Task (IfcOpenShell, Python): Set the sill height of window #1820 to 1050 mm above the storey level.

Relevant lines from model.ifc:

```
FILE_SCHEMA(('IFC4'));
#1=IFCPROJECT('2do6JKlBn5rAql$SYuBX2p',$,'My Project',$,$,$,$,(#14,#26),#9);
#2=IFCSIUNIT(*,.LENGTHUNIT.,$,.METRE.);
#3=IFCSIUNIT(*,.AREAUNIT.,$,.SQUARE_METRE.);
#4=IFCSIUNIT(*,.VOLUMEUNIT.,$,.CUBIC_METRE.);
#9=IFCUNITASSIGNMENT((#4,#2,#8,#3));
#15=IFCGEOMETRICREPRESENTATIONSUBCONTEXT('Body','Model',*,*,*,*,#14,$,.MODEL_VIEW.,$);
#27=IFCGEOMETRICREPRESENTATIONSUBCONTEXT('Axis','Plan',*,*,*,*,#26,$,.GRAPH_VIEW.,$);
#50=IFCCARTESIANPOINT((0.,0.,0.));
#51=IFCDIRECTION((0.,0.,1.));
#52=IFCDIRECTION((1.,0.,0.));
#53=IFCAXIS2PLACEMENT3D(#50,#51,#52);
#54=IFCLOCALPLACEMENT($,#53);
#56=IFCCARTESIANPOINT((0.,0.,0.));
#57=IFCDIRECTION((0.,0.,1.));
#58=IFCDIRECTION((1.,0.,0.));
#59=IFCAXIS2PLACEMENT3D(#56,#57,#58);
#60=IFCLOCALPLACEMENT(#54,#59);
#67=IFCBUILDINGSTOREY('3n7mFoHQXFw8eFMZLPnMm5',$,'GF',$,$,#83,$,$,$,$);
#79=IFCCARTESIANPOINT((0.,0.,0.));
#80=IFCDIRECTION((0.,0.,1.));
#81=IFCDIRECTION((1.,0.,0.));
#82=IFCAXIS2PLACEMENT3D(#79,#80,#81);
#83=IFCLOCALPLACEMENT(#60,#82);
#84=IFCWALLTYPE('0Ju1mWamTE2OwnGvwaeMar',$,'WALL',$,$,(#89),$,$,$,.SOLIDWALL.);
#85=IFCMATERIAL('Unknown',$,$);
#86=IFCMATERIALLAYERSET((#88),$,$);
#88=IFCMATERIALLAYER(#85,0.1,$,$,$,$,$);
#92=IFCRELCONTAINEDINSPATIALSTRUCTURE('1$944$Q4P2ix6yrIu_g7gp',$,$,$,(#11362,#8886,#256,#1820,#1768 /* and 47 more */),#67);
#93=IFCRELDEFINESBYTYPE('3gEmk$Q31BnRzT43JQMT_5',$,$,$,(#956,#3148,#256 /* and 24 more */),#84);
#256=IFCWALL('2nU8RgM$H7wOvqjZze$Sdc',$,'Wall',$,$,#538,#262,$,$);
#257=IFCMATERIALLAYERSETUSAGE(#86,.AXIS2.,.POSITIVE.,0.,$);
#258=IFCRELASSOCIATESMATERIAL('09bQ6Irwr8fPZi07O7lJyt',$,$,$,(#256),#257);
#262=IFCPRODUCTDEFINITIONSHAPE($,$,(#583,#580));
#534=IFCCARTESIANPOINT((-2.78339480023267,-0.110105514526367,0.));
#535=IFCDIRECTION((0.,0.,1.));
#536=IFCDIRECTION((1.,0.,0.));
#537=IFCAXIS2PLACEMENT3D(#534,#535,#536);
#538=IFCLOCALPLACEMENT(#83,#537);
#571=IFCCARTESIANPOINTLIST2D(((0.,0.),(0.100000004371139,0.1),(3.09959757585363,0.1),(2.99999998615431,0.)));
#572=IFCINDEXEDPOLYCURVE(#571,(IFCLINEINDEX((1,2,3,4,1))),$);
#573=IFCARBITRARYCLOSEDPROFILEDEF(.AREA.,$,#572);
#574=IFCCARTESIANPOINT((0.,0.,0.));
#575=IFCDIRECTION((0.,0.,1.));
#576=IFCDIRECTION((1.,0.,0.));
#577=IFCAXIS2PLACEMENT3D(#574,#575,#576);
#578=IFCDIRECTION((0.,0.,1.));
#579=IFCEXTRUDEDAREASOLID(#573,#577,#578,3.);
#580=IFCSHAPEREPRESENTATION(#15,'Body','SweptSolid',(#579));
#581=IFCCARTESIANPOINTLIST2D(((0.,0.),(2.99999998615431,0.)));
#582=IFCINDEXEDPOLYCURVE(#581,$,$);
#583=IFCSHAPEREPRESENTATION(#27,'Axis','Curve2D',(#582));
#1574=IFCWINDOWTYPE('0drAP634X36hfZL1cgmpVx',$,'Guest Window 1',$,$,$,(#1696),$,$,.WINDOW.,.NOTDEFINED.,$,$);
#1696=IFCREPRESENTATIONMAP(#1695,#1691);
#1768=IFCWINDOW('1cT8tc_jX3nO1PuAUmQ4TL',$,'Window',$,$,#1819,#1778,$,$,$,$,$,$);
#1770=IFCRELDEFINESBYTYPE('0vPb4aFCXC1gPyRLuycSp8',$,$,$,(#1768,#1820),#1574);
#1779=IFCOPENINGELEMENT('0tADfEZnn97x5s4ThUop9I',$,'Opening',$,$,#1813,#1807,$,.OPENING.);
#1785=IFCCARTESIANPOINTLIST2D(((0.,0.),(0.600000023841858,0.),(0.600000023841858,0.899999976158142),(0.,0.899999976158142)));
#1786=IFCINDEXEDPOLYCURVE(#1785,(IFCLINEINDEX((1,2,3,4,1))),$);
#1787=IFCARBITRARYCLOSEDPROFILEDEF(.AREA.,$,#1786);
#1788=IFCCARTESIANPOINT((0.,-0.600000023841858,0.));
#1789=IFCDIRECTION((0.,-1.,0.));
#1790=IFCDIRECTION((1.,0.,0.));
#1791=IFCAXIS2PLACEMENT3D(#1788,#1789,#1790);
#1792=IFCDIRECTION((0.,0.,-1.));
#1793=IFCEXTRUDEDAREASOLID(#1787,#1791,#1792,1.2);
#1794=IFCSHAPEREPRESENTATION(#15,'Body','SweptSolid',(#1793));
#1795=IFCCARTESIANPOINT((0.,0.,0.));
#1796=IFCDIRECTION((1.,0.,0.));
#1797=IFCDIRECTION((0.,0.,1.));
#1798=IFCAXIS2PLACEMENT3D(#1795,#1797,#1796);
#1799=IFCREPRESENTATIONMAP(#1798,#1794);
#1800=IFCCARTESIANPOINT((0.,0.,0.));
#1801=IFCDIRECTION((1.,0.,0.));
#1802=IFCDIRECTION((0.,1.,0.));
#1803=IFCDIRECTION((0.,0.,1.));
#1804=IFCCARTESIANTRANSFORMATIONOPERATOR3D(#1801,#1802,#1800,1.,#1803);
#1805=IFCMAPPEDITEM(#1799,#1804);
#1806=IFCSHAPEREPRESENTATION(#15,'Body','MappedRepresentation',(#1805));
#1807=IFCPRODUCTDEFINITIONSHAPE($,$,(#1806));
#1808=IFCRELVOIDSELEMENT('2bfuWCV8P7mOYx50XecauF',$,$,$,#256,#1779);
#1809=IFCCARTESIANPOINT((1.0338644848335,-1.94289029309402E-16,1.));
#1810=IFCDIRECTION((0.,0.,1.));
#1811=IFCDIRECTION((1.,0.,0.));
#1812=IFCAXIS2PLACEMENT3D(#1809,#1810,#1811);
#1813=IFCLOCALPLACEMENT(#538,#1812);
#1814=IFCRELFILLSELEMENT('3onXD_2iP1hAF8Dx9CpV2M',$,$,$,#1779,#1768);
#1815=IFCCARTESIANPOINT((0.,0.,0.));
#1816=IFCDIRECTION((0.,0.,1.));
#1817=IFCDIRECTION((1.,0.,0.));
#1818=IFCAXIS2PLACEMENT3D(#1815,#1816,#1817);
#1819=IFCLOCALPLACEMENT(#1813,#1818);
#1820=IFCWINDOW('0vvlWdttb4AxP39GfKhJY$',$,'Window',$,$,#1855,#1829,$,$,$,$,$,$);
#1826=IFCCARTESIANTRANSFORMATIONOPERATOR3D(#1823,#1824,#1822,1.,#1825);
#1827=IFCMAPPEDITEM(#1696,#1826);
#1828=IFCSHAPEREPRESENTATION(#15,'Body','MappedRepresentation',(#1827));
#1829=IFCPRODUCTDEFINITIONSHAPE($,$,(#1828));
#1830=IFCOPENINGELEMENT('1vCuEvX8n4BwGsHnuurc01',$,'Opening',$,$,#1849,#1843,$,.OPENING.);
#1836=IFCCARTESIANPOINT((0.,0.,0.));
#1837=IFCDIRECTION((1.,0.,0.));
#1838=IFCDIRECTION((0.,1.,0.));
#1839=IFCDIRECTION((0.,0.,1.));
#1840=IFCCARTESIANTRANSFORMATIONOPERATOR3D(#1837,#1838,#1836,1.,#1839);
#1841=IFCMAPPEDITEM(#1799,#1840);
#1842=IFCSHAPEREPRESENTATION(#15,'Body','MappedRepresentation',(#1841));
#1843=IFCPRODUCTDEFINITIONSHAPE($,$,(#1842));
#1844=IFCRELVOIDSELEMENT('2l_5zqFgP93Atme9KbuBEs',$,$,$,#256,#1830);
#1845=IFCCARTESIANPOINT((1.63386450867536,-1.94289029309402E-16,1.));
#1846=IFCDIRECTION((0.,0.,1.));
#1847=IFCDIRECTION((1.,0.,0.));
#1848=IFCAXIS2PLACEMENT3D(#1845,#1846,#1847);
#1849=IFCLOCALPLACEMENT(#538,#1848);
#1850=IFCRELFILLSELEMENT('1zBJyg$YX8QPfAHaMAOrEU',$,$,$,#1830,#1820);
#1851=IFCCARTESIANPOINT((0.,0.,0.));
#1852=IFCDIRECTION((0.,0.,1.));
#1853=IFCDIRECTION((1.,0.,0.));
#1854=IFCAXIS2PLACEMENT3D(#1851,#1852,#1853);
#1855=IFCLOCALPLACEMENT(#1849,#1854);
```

```python
import numpy as np
import ifcopenshell
import ifcopenshell.api.geometry
import ifcopenshell.geom
import ifcopenshell.util.element
import ifcopenshell.util.placement
import ifcopenshell.util.shape
import ifcopenshell.util.unit

model = ifcopenshell.open("model.ifc")
unit_scale = ifcopenshell.util.unit.calculate_unit_scale(model)

window = model.by_guid("0vvlWdttb4AxP39GfKhJY$")
opening = window.FillsVoids[0].RelatingOpeningElement
storey = ifcopenshell.util.element.get_container(window, ifc_class="IfcBuildingStorey")
level = ifcopenshell.util.placement.get_local_placement(storey.ObjectPlacement)[2, 3]

# The opening's origin need not be at the sill, so measure its lowest point.
shape = ifcopenshell.geom.create_shape(ifcopenshell.geom.settings(), opening)
bottom = ifcopenshell.util.shape.get_shape_bottom_elevation(shape, shape.geometry) / unit_scale
dz = level + 1.05 / unit_scale - bottom

shift = np.array([0.0, 0.0, dz])
# The window is placed relative to its opening, so it follows when the opening moves.
matrix = ifcopenshell.util.placement.get_local_placement(opening.ObjectPlacement)
matrix[:3, 3] += shift
ifcopenshell.api.geometry.edit_object_placement(
    model, product=opening, matrix=matrix, is_si=False, should_transform_children=True
)

print(f"moved by {dz * unit_scale:+.3f} m")

model.write("model_v2.ifc")
```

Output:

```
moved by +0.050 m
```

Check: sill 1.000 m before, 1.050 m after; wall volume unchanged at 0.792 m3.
